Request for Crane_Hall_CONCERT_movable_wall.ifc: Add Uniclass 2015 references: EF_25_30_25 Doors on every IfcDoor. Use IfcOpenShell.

First a look at what the model holds.

```python
import ifcopenshell

model = ifcopenshell.open("Crane_Hall_CONCERT_movable_wall.ifc")
print(model.schema)
print("classifications:", [c.Name for c in model.by_type("IfcClassification")])
for ifc_class in ("IfcDoor", "IfcRoof", "IfcStair", "IfcWall", "IfcWindow"):
    print(ifc_class, len(model.by_type(ifc_class)))
```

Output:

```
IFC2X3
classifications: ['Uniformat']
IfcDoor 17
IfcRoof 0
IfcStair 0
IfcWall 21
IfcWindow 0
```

```python
import ifcopenshell
import ifcopenshell.api.classification

model = ifcopenshell.open("Crane_Hall_CONCERT_movable_wall.ifc")

# IFC2X3 requires Source and Edition and has no link from the project to the system.
system = model.create_entity("IfcClassification", Source="NBS", Edition="2015", Name="Uniclass 2015")

codes = {
    "IfcDoor": ("EF_25_30_25", "Doors"),
}
for ifc_class, (code, name) in codes.items():
    products = model.by_type(ifc_class)
    ifcopenshell.api.classification.add_reference(
        model, products=products, classification=system, identification=code, name=name
    )
    print(code, len(products))

model.write("Crane_Hall_CONCERT_movable_wall_updated.ifc")
```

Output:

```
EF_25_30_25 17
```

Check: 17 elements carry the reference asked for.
